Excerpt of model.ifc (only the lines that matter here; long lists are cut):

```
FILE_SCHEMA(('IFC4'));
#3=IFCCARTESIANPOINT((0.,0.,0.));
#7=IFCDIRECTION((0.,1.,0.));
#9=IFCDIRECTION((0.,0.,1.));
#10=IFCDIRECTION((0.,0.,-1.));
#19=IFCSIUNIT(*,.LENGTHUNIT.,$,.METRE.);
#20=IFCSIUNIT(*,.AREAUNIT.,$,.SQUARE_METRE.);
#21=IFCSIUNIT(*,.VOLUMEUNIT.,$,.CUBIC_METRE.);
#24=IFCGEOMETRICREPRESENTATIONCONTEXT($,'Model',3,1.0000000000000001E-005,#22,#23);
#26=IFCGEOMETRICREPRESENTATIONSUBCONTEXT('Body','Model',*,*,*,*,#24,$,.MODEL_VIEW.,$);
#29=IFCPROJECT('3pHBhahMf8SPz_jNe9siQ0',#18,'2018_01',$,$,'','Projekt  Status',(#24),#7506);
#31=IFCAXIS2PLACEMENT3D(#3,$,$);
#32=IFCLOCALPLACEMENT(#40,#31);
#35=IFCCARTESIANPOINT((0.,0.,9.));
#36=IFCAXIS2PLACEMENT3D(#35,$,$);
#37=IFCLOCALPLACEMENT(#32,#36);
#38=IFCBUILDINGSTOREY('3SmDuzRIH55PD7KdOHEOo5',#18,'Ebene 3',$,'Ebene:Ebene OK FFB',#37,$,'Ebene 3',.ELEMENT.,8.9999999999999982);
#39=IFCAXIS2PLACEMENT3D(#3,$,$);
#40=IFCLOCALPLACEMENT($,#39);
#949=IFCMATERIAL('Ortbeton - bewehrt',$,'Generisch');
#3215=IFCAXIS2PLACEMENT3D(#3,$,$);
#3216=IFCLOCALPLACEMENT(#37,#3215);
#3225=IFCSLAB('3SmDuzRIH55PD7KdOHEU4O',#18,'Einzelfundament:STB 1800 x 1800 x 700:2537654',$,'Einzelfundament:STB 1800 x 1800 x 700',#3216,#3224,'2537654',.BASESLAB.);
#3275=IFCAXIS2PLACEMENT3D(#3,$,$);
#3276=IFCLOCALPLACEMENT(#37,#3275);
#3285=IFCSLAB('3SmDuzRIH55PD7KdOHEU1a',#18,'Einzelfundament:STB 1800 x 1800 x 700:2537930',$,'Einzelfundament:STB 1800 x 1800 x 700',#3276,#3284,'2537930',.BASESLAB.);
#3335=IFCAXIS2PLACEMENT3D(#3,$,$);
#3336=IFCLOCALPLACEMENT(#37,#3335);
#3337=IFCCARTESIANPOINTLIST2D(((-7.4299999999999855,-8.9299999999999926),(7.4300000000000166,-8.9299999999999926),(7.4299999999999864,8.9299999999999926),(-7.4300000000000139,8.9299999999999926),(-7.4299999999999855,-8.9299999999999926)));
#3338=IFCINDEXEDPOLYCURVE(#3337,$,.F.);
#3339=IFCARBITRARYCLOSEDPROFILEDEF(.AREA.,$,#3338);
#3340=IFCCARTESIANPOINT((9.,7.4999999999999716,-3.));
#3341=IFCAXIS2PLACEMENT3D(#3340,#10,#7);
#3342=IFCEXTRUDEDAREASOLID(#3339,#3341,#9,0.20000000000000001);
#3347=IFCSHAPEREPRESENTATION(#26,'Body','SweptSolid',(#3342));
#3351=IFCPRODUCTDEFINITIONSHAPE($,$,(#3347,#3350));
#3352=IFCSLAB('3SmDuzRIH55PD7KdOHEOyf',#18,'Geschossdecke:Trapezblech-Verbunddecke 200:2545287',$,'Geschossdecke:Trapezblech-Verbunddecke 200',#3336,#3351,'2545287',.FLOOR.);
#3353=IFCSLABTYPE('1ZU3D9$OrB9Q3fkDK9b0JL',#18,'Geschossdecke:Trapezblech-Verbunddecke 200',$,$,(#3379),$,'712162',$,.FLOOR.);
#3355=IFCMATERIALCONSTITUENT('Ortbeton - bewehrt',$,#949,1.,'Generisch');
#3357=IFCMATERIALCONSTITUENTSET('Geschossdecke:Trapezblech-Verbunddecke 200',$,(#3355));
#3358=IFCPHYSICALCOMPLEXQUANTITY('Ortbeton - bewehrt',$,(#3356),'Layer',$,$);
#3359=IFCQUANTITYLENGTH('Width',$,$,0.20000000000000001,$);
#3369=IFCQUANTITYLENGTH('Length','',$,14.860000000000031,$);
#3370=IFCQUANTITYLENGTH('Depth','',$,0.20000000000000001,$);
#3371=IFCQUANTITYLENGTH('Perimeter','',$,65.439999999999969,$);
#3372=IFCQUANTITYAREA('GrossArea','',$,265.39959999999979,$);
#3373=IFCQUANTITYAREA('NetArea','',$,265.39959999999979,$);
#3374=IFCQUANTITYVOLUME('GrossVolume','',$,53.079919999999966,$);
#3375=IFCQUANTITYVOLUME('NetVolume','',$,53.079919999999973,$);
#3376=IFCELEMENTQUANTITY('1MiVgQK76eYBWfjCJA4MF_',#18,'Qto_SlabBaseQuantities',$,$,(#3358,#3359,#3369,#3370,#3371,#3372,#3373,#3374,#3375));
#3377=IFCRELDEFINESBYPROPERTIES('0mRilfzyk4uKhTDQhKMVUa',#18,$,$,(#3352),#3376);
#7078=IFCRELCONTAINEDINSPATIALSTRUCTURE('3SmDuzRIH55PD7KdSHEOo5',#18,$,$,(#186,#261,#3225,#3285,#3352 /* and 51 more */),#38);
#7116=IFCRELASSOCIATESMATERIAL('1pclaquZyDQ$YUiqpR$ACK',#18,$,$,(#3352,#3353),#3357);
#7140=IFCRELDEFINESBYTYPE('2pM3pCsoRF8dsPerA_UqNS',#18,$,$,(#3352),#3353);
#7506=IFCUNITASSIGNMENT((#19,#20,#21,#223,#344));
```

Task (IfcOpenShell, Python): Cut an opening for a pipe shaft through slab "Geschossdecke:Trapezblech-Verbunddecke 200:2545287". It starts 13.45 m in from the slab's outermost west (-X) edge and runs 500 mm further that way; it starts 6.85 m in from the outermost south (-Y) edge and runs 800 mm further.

```python
import numpy as np
import ifcopenshell
import ifcopenshell.api.feature
import ifcopenshell.api.geometry
import ifcopenshell.api.pset
import ifcopenshell.api.root
import ifcopenshell.geom
import ifcopenshell.util.element
import ifcopenshell.util.placement
import ifcopenshell.util.representation
import ifcopenshell.util.shape
import ifcopenshell.util.unit

model = ifcopenshell.open("model.ifc")
unit_scale = ifcopenshell.util.unit.calculate_unit_scale(model)
area_scale = ifcopenshell.util.unit.calculate_unit_scale(model, "AREAUNIT")
volume_scale = ifcopenshell.util.unit.calculate_unit_scale(model, "VOLUMEUNIT")
settings = ifcopenshell.geom.settings()


def volume(element):
    """Net volume in cubic metres, openings subtracted."""
    shape = ifcopenshell.geom.create_shape(settings, element)
    return ifcopenshell.util.shape.get_volume(shape.geometry)


slab = model.by_guid("3SmDuzRIH55PD7KdOHEOyf")
before = volume(slab)

# Extent in the slab's own axes, in metres. The edges named are its -X and -Y sides.
slab_shape = ifcopenshell.geom.create_shape(settings, slab)
vertices = ifcopenshell.util.shape.get_vertices(slab_shape.geometry)
x_min, y_min, bottom = vertices.min(axis=0)
top = vertices[:, 2].max()

opening = ifcopenshell.api.root.create_entity(model, ifc_class="IfcOpeningElement", name="Pipe shaft opening", predefined_type="OPENING")
context = ifcopenshell.util.representation.get_context(model, "Model", "Body", "MODEL_VIEW")
width, depth = 0.5, 0.8
outline = [(0.0, 0.0), (width, 0.0), (width, depth), (0.0, depth), (0.0, 0.0)]
# Overshoot both faces by 50 mm so the cut is clean.
shape = ifcopenshell.api.geometry.add_slab_representation(
    model, context=context, depth=top - bottom + 0.1, polyline=outline
)
ifcopenshell.api.geometry.assign_representation(model, product=opening, representation=shape)

matrix = ifcopenshell.util.placement.get_local_placement(slab.ObjectPlacement)
matrix[:, 3] = matrix @ np.append(np.array([x_min + 13.45, y_min + 6.85, bottom - 0.05]) / unit_scale, 1.0)
ifcopenshell.api.geometry.edit_object_placement(model, product=opening, matrix=matrix, is_si=False)
ifcopenshell.api.feature.add_feature(model, feature=opening, element=slab)

after = volume(slab)

# Update the slab's stored quantities.
qto = model.by_id(ifcopenshell.util.element.get_pset(slab, "Qto_SlabBaseQuantities", should_inherit=False)["id"])
ifcopenshell.api.pset.edit_qto(model, qto=qto, properties={
    "NetArea": after / (top - bottom) / area_scale,
    "NetVolume": after / volume_scale,
})

print(f"slab volume {before:.3f} -> {after:.3f} m3")

model.write("model_updated.ifc")
```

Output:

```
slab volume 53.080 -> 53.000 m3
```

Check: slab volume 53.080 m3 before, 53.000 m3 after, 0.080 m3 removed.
